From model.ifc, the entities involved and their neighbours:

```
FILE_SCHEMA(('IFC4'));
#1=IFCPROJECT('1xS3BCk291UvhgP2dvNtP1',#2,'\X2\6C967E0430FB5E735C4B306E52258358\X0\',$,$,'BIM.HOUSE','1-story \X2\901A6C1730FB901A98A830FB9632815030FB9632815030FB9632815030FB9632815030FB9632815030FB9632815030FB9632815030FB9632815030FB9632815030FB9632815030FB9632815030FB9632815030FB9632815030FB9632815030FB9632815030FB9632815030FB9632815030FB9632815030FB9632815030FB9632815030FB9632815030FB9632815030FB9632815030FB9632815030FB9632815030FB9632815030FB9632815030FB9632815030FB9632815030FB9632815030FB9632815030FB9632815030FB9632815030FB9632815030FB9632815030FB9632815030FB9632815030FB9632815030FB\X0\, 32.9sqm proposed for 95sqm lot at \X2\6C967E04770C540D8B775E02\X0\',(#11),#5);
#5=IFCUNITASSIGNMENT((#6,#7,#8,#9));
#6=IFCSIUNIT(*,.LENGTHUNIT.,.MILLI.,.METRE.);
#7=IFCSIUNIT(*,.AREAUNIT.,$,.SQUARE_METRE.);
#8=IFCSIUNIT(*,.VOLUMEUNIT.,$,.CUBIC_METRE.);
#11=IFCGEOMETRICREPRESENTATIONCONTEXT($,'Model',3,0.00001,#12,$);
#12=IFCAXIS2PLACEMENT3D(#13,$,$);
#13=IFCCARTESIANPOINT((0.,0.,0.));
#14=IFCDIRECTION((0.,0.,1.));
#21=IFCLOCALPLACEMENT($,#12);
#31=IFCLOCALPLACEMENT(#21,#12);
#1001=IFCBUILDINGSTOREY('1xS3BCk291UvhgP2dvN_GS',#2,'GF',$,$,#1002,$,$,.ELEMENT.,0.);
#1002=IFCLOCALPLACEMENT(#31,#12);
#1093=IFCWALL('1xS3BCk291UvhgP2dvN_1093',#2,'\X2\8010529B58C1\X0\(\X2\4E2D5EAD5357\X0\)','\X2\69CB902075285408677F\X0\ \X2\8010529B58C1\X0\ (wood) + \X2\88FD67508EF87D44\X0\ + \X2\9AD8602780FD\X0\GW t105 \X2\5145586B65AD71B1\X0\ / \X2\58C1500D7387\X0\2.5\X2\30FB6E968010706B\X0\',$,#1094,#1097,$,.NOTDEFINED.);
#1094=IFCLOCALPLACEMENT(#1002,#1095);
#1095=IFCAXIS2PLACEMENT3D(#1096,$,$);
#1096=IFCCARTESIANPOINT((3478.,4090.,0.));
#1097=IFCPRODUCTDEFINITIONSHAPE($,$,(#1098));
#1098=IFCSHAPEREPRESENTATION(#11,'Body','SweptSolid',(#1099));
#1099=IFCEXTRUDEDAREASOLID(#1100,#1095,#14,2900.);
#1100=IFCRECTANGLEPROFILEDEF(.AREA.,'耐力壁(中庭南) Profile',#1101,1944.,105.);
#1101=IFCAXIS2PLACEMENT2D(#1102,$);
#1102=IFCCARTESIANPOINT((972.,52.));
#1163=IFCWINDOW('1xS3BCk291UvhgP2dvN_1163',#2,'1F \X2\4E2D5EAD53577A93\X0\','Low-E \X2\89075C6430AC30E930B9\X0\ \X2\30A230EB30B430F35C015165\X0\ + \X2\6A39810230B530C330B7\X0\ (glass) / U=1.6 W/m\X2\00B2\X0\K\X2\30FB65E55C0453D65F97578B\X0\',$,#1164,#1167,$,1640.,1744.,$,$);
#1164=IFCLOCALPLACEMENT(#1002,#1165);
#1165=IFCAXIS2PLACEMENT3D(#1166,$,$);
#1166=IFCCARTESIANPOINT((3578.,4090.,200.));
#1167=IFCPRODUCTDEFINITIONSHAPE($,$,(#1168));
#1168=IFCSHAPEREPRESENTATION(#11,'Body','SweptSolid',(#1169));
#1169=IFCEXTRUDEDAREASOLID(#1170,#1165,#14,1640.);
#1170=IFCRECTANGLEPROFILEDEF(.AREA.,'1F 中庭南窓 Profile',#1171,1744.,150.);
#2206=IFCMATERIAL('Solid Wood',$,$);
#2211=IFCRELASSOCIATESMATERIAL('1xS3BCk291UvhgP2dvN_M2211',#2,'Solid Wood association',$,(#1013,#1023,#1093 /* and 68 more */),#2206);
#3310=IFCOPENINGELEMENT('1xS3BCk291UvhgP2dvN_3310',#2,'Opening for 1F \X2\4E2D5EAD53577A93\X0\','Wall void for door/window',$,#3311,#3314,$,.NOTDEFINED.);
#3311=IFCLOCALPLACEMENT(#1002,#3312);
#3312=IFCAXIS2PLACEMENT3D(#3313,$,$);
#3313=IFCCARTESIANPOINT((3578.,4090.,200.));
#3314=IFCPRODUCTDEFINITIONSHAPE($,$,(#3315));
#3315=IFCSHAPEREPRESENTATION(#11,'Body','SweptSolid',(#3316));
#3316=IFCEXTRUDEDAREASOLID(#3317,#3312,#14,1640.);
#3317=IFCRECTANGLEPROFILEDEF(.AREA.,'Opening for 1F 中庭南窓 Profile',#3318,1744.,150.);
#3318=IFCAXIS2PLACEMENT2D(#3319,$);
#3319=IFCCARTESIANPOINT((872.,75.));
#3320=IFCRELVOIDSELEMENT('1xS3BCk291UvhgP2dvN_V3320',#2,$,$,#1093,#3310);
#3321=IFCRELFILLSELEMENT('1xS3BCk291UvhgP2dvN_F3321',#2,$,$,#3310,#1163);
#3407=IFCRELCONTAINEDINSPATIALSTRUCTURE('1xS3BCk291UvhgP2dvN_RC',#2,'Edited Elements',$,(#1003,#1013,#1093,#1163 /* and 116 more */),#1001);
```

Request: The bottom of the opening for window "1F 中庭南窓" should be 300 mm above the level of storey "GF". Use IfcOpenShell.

```python
import numpy as np
import ifcopenshell
import ifcopenshell.api.geometry
import ifcopenshell.geom
import ifcopenshell.util.element
import ifcopenshell.util.placement
import ifcopenshell.util.shape
import ifcopenshell.util.unit

model = ifcopenshell.open("model.ifc")
unit_scale = ifcopenshell.util.unit.calculate_unit_scale(model)

window = model.by_id(1163)
opening = window.FillsVoids[0].RelatingOpeningElement
storey = ifcopenshell.util.element.get_container(window, ifc_class="IfcBuildingStorey")
level = ifcopenshell.util.placement.get_local_placement(storey.ObjectPlacement)[2, 3]

# The opening's origin need not be at the sill, so measure its lowest point.
shape = ifcopenshell.geom.create_shape(ifcopenshell.geom.settings(), opening)
bottom = ifcopenshell.util.shape.get_shape_bottom_elevation(shape, shape.geometry) / unit_scale
dz = level + 0.3 / unit_scale - bottom

shift = np.array([0.0, 0.0, dz])
# The window is not placed relative to its opening, so move both.
for product in (opening, window):
    matrix = ifcopenshell.util.placement.get_local_placement(product.ObjectPlacement)
    matrix[:3, 3] += shift
    ifcopenshell.api.geometry.edit_object_placement(model, product=product, matrix=matrix, is_si=False)

print(f"moved by {dz * unit_scale:+.3f} m")

model.write("model_updated.ifc")
```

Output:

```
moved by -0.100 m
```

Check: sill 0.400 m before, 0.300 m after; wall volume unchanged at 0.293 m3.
